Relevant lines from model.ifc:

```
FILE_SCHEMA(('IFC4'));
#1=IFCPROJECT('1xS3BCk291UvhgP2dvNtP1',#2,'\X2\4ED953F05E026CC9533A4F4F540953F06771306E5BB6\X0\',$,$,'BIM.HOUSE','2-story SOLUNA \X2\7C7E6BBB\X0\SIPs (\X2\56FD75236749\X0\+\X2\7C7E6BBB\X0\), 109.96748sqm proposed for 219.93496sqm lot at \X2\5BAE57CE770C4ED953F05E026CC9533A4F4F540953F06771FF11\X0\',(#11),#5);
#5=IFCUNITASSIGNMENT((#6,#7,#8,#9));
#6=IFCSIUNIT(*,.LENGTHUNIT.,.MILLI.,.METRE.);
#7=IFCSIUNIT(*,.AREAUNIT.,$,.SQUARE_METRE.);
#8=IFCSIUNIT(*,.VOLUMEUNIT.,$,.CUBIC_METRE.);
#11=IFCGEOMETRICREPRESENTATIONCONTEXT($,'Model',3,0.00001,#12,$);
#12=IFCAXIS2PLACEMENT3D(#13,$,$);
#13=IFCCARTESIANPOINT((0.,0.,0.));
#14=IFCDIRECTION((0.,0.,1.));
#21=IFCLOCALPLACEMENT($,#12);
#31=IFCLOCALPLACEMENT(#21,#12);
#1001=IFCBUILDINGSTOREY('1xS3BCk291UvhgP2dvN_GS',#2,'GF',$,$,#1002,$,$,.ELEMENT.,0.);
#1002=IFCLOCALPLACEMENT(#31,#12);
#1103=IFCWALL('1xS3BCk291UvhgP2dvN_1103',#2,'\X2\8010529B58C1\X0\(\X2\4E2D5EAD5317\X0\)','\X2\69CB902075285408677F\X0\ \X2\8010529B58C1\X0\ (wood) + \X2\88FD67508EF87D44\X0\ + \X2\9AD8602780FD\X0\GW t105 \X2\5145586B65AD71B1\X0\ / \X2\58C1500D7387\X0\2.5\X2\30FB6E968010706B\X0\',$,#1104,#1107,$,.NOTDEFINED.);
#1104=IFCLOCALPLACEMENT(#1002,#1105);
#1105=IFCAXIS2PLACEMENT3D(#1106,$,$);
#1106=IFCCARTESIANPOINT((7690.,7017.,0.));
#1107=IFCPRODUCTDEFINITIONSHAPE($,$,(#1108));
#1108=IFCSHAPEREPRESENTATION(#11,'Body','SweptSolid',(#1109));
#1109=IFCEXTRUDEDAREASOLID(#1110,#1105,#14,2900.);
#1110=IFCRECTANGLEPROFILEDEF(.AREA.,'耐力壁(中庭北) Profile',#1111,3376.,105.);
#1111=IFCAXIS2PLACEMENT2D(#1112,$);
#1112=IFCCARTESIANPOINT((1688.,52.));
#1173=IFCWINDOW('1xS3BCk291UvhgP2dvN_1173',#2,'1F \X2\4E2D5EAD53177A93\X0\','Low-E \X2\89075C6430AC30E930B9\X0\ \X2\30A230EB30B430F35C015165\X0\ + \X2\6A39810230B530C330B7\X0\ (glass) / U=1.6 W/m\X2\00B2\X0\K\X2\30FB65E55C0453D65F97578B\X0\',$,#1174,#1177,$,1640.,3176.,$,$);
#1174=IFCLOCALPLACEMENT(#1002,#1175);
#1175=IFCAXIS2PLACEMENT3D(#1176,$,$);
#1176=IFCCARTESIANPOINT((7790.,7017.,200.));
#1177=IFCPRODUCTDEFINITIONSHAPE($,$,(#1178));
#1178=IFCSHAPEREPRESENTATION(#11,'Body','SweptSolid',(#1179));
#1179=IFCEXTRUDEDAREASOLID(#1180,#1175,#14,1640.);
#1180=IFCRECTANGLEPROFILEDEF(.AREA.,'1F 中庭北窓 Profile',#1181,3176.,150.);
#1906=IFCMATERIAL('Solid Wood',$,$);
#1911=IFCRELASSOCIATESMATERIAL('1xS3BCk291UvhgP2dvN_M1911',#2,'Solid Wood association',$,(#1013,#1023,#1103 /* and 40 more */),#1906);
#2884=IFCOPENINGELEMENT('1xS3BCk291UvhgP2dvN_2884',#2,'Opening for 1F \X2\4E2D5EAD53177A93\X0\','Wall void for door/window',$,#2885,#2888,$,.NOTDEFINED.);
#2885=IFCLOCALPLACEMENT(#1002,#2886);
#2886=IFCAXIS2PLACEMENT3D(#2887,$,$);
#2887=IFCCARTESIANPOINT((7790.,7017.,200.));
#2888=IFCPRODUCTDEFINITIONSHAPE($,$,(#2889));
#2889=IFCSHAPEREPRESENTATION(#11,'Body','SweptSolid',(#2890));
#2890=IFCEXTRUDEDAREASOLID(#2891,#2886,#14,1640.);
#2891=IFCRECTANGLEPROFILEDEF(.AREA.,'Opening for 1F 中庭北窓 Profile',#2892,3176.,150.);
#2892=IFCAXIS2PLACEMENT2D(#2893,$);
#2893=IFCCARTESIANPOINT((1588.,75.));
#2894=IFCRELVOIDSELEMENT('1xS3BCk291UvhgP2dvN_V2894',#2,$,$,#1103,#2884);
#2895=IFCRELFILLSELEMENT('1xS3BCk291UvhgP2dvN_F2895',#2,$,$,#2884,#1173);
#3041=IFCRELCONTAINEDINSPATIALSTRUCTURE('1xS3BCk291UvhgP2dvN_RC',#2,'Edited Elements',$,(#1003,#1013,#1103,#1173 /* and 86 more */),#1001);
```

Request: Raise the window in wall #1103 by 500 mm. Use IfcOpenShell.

```python
import numpy as np
import ifcopenshell
import ifcopenshell.api.geometry
import ifcopenshell.util.placement
import ifcopenshell.util.unit

model = ifcopenshell.open("model.ifc")
unit_scale = ifcopenshell.util.unit.calculate_unit_scale(model)

window = model.by_guid("1xS3BCk291UvhgP2dvN_1173")
opening = window.FillsVoids[0].RelatingOpeningElement
dz = 500.0

shift = np.array([0.0, 0.0, dz])
# The window is not placed relative to its opening, so move both.
for product in (opening, window):
    matrix = ifcopenshell.util.placement.get_local_placement(product.ObjectPlacement)
    matrix[:3, 3] += shift
    ifcopenshell.api.geometry.edit_object_placement(model, product=product, matrix=matrix, is_si=False)

print(f"moved by {dz * unit_scale:+.3f} m")

model.write("model_edited.ifc")
```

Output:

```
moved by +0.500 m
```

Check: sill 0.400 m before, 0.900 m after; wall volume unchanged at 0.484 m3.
